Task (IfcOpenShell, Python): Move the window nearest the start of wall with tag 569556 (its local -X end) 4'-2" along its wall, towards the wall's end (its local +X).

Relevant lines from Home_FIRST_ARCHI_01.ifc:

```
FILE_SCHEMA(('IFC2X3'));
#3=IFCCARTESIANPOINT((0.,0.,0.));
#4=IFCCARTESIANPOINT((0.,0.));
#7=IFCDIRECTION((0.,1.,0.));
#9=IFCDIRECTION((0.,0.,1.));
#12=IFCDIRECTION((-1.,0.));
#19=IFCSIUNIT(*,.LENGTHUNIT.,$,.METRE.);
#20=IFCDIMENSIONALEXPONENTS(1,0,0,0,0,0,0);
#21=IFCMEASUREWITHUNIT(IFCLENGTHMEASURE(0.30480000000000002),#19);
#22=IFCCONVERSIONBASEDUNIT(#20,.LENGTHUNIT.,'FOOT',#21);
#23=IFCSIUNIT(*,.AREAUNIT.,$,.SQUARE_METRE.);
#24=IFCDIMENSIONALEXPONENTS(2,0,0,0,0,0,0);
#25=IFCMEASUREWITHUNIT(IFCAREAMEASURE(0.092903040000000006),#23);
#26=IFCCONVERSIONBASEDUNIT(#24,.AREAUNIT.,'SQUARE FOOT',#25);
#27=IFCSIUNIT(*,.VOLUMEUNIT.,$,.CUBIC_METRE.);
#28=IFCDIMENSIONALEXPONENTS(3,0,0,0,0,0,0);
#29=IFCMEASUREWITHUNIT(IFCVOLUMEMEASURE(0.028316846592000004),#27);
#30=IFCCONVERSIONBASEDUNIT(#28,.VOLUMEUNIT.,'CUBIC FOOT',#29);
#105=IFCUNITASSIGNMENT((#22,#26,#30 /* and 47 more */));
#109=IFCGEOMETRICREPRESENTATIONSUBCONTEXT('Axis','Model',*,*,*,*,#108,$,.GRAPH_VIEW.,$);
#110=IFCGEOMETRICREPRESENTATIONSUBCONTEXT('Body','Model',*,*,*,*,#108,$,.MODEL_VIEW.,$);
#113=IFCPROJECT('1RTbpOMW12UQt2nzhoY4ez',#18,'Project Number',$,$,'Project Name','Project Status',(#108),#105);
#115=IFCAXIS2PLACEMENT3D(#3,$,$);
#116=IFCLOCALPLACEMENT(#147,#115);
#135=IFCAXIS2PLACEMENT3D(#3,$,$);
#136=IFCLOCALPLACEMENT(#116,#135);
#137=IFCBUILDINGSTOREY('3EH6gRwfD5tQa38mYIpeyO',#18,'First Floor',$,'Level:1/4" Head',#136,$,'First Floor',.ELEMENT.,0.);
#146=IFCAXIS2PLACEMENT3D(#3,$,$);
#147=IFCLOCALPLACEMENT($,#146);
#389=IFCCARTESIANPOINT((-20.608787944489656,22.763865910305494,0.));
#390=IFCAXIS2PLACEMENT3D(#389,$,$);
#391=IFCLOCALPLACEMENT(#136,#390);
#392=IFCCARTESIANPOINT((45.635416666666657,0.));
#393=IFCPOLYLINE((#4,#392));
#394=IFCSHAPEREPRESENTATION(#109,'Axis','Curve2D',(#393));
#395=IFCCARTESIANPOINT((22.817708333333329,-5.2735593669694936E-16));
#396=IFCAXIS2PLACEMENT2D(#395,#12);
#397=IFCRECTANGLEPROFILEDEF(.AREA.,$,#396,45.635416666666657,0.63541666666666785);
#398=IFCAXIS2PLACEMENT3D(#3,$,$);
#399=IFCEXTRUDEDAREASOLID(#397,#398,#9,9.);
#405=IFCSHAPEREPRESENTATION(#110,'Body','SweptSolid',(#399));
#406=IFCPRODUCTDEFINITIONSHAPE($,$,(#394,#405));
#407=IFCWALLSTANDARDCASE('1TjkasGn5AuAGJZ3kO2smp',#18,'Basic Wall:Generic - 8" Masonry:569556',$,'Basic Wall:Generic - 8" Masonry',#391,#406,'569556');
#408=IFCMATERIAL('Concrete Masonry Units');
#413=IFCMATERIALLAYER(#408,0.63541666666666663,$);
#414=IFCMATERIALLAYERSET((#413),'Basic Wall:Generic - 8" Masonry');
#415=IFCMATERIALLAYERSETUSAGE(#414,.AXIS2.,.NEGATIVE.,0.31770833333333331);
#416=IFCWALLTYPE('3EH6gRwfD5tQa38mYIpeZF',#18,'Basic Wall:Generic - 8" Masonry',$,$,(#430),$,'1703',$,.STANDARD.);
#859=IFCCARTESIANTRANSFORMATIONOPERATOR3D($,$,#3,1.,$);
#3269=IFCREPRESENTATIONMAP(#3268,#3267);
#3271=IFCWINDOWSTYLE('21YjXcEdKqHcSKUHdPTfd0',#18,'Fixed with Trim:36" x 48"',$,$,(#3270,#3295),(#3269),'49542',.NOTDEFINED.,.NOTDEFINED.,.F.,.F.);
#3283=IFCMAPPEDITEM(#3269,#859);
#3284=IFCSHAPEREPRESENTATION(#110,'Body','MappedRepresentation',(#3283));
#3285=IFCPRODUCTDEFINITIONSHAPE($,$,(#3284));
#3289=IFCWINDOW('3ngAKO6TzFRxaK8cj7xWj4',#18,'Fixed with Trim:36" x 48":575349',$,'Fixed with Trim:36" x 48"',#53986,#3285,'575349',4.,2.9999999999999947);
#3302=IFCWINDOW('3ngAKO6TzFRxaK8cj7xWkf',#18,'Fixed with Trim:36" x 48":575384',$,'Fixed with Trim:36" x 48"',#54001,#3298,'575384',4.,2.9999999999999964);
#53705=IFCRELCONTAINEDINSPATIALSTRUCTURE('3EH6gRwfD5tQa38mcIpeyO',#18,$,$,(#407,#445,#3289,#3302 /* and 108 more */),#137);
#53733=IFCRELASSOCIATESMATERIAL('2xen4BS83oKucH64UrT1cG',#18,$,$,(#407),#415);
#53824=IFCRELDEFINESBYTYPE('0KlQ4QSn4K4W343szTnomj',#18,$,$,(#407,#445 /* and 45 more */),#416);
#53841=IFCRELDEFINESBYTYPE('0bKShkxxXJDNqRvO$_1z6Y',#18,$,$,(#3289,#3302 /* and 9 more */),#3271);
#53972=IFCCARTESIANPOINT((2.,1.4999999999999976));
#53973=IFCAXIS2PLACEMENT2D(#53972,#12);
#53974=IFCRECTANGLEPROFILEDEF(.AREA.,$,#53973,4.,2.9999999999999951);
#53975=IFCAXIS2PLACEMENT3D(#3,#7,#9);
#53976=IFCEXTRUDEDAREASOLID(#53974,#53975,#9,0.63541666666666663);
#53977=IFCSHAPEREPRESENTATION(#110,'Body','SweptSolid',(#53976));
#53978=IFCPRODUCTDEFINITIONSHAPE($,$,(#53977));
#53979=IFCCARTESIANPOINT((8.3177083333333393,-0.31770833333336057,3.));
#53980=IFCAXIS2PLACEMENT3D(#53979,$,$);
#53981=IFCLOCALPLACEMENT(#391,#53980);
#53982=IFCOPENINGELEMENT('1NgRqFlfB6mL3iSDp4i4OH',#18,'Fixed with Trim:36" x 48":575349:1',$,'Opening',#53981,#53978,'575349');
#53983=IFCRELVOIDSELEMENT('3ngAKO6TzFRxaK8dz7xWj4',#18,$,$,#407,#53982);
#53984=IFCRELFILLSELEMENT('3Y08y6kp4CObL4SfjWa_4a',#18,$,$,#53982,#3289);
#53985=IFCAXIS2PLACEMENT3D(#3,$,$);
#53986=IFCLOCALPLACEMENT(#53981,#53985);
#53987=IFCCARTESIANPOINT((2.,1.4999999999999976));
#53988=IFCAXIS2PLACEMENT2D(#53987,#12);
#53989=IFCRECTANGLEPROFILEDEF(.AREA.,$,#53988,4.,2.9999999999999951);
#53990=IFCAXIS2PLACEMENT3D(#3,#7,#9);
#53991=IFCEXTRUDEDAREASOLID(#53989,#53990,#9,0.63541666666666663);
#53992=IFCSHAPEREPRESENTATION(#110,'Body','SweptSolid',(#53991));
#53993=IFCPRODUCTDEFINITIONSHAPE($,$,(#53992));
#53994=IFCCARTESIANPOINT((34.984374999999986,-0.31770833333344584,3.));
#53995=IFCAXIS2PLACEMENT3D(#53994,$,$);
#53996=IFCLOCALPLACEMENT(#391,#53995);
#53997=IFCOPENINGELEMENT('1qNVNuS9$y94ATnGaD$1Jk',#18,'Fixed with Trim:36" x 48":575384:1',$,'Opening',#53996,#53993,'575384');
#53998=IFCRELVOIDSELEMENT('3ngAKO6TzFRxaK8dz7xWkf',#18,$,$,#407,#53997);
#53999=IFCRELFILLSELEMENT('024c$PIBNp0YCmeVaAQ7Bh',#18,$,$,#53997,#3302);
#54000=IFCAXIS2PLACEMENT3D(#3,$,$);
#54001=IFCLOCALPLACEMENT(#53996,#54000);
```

```python
import ifcopenshell
import ifcopenshell.api.geometry
import ifcopenshell.util.placement
import ifcopenshell.util.unit

model = ifcopenshell.open("Home_FIRST_ARCHI_01.ifc")
unit_scale = ifcopenshell.util.unit.calculate_unit_scale(model)

window = model.by_guid("3ngAKO6TzFRxaK8cj7xWj4")
opening = window.FillsVoids[0].RelatingOpeningElement
wall = opening.VoidsElements[0].RelatingBuildingElement

wall_matrix = ifcopenshell.util.placement.get_local_placement(wall.ObjectPlacement)
shift = wall_matrix[:3, 0] * 50 * 0.0254 / unit_scale
before = ifcopenshell.util.placement.get_local_placement(window.ObjectPlacement)[:3, 3].copy()

# The window is placed relative to its opening, so it follows when the opening moves.
matrix = ifcopenshell.util.placement.get_local_placement(opening.ObjectPlacement)
matrix[:3, 3] += shift
ifcopenshell.api.geometry.edit_object_placement(
    model, product=opening, matrix=matrix, is_si=False, should_transform_children=True
)

after = ifcopenshell.util.placement.get_local_placement(window.ObjectPlacement)[:3, 3]
print("window moved by", (after - before).round(3) + 0.0)

model.write("Home_FIRST_ARCHI_01_v2.ifc")
```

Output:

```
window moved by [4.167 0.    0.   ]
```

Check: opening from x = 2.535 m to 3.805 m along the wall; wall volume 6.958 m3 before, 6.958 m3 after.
